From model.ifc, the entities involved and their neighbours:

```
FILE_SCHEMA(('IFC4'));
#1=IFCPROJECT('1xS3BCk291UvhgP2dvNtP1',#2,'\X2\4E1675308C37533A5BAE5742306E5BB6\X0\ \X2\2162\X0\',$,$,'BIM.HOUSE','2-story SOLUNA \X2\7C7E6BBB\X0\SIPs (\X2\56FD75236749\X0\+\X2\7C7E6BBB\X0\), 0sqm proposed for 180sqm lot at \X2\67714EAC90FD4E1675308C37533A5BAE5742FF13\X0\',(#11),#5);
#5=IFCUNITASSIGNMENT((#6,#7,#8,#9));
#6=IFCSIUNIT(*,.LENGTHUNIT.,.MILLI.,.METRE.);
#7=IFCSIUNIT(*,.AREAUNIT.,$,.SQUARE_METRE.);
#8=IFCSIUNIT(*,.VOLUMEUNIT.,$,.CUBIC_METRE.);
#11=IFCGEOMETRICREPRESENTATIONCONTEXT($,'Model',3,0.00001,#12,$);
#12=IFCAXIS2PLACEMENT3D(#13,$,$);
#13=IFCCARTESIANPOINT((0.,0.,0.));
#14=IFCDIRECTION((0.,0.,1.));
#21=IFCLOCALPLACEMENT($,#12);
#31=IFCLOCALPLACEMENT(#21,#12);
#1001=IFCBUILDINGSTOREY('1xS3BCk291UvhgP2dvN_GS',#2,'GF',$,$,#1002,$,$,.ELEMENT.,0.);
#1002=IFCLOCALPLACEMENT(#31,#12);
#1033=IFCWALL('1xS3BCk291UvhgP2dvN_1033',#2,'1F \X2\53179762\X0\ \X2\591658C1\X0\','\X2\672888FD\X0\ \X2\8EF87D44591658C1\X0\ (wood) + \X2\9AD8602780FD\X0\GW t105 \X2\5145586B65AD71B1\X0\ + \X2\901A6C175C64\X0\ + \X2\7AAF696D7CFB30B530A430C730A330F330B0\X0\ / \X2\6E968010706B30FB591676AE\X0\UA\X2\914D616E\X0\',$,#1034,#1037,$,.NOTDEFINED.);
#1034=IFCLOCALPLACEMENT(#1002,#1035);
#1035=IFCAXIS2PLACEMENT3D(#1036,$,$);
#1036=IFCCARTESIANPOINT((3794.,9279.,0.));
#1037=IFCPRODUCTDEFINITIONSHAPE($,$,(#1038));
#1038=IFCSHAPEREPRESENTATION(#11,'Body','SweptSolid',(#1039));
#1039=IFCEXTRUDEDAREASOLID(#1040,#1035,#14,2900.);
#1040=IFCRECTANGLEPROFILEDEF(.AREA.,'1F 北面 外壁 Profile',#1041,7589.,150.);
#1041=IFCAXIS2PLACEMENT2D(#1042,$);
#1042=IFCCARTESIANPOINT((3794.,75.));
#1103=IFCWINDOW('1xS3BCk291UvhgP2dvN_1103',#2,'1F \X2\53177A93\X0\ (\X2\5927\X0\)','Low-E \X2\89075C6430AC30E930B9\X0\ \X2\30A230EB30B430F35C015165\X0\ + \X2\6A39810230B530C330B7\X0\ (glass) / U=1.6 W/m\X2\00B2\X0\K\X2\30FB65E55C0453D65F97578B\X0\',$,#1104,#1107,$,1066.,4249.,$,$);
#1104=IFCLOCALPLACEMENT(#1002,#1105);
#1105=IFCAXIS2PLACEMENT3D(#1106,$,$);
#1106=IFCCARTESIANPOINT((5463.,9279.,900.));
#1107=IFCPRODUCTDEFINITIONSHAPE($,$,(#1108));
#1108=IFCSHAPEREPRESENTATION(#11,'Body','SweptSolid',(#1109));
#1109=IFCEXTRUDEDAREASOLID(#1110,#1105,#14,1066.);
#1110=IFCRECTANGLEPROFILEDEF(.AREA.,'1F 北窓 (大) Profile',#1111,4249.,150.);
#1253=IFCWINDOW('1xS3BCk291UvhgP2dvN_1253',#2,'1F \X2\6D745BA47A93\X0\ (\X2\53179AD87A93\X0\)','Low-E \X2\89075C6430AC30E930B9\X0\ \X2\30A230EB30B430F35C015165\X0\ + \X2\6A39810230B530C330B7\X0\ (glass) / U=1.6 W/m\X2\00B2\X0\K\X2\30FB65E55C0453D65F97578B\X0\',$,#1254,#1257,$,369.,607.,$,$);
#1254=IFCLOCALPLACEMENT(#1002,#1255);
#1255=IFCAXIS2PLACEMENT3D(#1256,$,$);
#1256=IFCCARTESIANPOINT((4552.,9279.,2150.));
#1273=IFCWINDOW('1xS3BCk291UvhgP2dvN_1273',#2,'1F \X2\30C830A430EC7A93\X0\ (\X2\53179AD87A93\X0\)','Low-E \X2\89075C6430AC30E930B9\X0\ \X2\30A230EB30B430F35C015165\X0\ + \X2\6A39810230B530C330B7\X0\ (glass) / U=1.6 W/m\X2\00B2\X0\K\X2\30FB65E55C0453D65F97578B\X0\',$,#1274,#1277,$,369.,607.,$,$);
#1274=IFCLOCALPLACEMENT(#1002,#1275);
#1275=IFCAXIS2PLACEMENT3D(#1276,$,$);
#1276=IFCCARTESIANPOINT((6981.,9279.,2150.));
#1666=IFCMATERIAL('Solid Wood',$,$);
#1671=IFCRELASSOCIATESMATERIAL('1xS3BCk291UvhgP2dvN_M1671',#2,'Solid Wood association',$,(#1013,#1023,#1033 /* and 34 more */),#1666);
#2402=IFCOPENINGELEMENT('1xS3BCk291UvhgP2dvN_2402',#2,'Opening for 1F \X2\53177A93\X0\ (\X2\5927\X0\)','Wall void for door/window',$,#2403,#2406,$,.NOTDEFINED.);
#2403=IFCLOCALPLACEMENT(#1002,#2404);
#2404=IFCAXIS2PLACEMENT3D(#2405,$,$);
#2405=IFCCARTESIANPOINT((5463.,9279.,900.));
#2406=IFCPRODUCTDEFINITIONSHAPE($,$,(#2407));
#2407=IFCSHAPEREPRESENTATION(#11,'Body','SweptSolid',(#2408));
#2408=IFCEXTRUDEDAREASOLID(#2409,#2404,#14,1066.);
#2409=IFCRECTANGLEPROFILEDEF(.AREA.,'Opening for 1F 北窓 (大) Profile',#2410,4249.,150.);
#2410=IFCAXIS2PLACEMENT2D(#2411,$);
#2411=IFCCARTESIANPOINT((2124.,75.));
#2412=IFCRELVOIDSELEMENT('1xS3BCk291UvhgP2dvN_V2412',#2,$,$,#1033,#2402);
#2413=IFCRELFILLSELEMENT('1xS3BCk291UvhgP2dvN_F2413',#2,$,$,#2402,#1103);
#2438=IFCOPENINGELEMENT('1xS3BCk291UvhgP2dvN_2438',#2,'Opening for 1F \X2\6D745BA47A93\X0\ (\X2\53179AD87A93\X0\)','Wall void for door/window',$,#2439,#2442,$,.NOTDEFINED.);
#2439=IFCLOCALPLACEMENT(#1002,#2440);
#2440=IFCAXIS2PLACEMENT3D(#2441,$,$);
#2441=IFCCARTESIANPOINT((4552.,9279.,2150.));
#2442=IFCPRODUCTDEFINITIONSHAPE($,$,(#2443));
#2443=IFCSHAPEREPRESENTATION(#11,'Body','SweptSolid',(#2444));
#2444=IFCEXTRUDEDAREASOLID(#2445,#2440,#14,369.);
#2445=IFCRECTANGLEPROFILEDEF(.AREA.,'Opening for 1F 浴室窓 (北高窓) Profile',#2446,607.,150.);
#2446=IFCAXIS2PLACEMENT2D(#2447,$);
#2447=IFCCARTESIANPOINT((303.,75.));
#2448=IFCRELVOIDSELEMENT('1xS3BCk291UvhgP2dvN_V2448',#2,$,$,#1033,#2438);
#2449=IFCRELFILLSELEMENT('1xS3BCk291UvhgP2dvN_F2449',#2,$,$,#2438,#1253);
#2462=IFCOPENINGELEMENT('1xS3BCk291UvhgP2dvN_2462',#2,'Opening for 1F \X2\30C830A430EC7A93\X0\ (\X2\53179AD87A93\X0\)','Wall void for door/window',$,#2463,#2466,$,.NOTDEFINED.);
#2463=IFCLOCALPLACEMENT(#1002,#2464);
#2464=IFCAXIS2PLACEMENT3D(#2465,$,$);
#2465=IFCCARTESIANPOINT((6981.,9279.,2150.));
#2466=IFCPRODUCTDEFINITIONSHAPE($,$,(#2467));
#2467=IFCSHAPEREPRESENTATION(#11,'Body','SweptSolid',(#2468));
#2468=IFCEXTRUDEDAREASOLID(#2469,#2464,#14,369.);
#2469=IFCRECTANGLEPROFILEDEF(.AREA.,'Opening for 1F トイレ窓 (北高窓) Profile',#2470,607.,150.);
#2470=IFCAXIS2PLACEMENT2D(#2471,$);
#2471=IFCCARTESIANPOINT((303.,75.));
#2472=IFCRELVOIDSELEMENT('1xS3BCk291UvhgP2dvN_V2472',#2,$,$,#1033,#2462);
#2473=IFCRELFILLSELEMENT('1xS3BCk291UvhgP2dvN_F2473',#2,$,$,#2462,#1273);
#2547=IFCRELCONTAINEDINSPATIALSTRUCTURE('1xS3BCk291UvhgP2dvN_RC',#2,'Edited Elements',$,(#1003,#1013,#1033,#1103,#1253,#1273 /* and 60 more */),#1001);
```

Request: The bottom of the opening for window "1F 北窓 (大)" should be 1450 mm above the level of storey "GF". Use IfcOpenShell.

```python
import numpy as np
import ifcopenshell
import ifcopenshell.api.geometry
import ifcopenshell.geom
import ifcopenshell.util.element
import ifcopenshell.util.placement
import ifcopenshell.util.shape
import ifcopenshell.util.unit

model = ifcopenshell.open("model.ifc")
unit_scale = ifcopenshell.util.unit.calculate_unit_scale(model)

window = model.by_id(1103)
opening = window.FillsVoids[0].RelatingOpeningElement
storey = ifcopenshell.util.element.get_container(window, ifc_class="IfcBuildingStorey")
level = ifcopenshell.util.placement.get_local_placement(storey.ObjectPlacement)[2, 3]

# The opening's origin need not be at the sill, so measure its lowest point.
shape = ifcopenshell.geom.create_shape(ifcopenshell.geom.settings(), opening)
bottom = ifcopenshell.util.shape.get_shape_bottom_elevation(shape, shape.geometry) / unit_scale
dz = level + 1.45 / unit_scale - bottom

shift = np.array([0.0, 0.0, dz])
# The window is not placed relative to its opening, so move both.
for product in (opening, window):
    matrix = ifcopenshell.util.placement.get_local_placement(product.ObjectPlacement)
    matrix[:3, 3] += shift
    ifcopenshell.api.geometry.edit_object_placement(model, product=product, matrix=matrix, is_si=False)

print(f"moved by {dz * unit_scale:+.3f} m")

model.write("model_updated.ifc")
```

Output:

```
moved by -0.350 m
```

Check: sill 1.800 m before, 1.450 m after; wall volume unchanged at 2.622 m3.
